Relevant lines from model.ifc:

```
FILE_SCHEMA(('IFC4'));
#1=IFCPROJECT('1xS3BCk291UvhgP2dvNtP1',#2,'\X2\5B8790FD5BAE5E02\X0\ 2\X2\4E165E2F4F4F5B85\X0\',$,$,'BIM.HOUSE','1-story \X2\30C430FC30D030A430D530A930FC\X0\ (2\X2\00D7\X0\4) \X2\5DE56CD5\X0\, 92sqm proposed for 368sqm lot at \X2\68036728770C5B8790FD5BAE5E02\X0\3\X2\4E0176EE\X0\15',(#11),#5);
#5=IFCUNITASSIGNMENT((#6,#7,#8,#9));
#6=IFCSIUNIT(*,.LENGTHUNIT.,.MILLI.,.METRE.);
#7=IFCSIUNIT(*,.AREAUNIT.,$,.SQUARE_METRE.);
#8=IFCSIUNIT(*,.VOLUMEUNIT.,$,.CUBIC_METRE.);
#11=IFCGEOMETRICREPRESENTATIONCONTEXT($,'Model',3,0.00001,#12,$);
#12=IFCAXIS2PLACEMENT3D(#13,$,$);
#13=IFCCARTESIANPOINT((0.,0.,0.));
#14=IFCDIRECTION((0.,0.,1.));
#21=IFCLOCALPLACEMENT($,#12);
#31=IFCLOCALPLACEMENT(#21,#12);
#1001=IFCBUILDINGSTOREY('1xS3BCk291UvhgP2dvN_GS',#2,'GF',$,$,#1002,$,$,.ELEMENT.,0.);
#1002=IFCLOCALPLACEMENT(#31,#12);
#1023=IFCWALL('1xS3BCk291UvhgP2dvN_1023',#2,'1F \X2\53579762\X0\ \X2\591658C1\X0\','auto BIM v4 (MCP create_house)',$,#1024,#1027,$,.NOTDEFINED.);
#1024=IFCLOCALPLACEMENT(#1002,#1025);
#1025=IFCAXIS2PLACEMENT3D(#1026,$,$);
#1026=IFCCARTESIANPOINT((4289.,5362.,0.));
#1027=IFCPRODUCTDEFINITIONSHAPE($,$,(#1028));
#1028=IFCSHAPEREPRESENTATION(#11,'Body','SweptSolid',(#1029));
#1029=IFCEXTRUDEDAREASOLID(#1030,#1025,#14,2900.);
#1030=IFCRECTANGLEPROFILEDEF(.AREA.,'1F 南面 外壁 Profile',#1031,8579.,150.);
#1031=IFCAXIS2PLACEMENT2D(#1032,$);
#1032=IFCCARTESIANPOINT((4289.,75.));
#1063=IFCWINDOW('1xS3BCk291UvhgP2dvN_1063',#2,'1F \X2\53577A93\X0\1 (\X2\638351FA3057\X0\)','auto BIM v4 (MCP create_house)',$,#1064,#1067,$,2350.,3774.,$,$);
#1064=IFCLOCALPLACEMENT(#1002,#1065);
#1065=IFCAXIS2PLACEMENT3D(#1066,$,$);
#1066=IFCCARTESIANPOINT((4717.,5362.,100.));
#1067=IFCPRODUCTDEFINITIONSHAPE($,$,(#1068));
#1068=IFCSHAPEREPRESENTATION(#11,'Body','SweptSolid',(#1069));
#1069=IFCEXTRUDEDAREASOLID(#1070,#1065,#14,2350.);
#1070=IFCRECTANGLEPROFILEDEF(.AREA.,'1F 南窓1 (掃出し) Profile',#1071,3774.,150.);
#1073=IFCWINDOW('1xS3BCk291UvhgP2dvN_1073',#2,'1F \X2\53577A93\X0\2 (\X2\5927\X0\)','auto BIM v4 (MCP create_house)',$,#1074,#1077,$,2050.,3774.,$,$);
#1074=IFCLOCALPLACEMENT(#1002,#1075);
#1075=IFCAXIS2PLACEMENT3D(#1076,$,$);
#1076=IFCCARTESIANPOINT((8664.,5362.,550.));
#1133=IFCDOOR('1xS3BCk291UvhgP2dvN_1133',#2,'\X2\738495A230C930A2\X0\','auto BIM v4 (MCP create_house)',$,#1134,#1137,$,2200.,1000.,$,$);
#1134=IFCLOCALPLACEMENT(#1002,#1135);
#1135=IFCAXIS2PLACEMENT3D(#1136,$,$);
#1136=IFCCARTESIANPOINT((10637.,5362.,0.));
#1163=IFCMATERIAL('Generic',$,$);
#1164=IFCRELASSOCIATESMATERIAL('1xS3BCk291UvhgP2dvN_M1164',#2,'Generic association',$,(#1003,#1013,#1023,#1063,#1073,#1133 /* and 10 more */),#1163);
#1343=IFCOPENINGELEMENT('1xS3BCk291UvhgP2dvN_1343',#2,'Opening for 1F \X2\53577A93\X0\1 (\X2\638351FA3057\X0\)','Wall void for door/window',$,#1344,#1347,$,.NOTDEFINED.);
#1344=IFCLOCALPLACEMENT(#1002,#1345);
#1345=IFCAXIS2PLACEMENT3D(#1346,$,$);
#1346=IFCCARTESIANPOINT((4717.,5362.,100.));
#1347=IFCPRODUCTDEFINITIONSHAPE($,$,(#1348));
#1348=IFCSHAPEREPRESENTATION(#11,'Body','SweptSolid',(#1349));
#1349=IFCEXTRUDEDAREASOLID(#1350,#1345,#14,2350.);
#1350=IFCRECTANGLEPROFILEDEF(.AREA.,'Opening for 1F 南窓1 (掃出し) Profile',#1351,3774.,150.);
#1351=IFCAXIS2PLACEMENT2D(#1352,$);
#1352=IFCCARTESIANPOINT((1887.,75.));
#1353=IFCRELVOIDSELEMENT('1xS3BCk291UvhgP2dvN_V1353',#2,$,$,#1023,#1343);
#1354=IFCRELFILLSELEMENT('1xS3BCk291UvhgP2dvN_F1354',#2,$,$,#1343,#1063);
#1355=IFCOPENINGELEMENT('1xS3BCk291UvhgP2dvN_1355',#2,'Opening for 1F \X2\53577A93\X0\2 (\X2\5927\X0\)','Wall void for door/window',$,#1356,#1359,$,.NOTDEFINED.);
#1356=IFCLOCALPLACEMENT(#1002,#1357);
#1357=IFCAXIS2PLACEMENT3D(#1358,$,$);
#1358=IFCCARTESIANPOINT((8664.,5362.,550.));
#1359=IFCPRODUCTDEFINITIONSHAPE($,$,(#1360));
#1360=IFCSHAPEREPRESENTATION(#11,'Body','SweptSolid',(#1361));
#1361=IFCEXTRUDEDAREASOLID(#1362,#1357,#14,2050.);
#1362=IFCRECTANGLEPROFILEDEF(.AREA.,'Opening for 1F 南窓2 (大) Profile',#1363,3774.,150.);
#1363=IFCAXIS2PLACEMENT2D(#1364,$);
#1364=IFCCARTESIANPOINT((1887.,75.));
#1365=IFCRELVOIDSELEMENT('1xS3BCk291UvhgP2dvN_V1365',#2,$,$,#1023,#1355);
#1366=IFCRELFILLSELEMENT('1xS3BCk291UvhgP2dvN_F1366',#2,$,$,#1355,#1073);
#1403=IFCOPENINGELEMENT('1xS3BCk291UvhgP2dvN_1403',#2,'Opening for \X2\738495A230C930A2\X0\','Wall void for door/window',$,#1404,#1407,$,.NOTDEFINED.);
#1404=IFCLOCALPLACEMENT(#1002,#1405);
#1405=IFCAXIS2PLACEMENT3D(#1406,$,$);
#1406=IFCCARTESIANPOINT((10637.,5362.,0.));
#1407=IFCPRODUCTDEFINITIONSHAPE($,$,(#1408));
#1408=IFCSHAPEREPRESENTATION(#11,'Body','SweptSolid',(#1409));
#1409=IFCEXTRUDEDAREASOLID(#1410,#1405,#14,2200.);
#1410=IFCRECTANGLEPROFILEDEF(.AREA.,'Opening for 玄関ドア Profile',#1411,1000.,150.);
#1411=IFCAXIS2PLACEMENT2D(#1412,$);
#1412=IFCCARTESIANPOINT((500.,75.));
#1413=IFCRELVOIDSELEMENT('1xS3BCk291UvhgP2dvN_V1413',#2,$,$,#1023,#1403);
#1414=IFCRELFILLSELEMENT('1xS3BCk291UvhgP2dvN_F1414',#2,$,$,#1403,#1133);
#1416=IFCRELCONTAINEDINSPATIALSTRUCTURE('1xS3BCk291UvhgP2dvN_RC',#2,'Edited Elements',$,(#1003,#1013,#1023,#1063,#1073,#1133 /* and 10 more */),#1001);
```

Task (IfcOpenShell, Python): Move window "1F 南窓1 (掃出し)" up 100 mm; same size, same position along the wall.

```python
import numpy as np
import ifcopenshell
import ifcopenshell.api.geometry
import ifcopenshell.util.placement
import ifcopenshell.util.unit

model = ifcopenshell.open("model.ifc")
unit_scale = ifcopenshell.util.unit.calculate_unit_scale(model)

window = model.by_guid("1xS3BCk291UvhgP2dvN_1063")
opening = window.FillsVoids[0].RelatingOpeningElement
dz = 100.0

shift = np.array([0.0, 0.0, dz])
# The window is not placed relative to its opening, so move both.
for product in (opening, window):
    matrix = ifcopenshell.util.placement.get_local_placement(product.ObjectPlacement)
    matrix[:3, 3] += shift
    ifcopenshell.api.geometry.edit_object_placement(model, product=product, matrix=matrix, is_si=False)

print(f"moved by {dz * unit_scale:+.3f} m")

model.write("model_v2.ifc")
```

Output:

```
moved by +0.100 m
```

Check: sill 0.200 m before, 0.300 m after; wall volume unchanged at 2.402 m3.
